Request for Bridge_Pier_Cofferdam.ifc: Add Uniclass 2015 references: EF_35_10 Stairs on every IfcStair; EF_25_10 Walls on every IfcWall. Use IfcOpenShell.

First a look at what the model holds.

```python
import ifcopenshell

model = ifcopenshell.open("Bridge_Pier_Cofferdam.ifc")
print(model.schema)
print("classifications:", [c.Name for c in model.by_type("IfcClassification")])
for ifc_class in ("IfcDoor", "IfcRoof", "IfcStair", "IfcWall", "IfcWindow"):
    print(ifc_class, len(model.by_type(ifc_class)))
```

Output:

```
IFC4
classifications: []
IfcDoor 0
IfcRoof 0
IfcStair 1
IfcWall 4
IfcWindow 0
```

```python
import ifcopenshell
import ifcopenshell.api.classification

model = ifcopenshell.open("Bridge_Pier_Cofferdam.ifc")

system = ifcopenshell.api.classification.add_classification(model, classification="Uniclass 2015")

codes = {
    "IfcStair": ("EF_35_10", "Stairs"),
    "IfcWall": ("EF_25_10", "Walls"),
}
for ifc_class, (code, name) in codes.items():
    products = model.by_type(ifc_class)
    ifcopenshell.api.classification.add_reference(
        model, products=products, classification=system, identification=code, name=name
    )
    print(code, len(products))

model.write("Bridge_Pier_Cofferdam_edited.ifc")
```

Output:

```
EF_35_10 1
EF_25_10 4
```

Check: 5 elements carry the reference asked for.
